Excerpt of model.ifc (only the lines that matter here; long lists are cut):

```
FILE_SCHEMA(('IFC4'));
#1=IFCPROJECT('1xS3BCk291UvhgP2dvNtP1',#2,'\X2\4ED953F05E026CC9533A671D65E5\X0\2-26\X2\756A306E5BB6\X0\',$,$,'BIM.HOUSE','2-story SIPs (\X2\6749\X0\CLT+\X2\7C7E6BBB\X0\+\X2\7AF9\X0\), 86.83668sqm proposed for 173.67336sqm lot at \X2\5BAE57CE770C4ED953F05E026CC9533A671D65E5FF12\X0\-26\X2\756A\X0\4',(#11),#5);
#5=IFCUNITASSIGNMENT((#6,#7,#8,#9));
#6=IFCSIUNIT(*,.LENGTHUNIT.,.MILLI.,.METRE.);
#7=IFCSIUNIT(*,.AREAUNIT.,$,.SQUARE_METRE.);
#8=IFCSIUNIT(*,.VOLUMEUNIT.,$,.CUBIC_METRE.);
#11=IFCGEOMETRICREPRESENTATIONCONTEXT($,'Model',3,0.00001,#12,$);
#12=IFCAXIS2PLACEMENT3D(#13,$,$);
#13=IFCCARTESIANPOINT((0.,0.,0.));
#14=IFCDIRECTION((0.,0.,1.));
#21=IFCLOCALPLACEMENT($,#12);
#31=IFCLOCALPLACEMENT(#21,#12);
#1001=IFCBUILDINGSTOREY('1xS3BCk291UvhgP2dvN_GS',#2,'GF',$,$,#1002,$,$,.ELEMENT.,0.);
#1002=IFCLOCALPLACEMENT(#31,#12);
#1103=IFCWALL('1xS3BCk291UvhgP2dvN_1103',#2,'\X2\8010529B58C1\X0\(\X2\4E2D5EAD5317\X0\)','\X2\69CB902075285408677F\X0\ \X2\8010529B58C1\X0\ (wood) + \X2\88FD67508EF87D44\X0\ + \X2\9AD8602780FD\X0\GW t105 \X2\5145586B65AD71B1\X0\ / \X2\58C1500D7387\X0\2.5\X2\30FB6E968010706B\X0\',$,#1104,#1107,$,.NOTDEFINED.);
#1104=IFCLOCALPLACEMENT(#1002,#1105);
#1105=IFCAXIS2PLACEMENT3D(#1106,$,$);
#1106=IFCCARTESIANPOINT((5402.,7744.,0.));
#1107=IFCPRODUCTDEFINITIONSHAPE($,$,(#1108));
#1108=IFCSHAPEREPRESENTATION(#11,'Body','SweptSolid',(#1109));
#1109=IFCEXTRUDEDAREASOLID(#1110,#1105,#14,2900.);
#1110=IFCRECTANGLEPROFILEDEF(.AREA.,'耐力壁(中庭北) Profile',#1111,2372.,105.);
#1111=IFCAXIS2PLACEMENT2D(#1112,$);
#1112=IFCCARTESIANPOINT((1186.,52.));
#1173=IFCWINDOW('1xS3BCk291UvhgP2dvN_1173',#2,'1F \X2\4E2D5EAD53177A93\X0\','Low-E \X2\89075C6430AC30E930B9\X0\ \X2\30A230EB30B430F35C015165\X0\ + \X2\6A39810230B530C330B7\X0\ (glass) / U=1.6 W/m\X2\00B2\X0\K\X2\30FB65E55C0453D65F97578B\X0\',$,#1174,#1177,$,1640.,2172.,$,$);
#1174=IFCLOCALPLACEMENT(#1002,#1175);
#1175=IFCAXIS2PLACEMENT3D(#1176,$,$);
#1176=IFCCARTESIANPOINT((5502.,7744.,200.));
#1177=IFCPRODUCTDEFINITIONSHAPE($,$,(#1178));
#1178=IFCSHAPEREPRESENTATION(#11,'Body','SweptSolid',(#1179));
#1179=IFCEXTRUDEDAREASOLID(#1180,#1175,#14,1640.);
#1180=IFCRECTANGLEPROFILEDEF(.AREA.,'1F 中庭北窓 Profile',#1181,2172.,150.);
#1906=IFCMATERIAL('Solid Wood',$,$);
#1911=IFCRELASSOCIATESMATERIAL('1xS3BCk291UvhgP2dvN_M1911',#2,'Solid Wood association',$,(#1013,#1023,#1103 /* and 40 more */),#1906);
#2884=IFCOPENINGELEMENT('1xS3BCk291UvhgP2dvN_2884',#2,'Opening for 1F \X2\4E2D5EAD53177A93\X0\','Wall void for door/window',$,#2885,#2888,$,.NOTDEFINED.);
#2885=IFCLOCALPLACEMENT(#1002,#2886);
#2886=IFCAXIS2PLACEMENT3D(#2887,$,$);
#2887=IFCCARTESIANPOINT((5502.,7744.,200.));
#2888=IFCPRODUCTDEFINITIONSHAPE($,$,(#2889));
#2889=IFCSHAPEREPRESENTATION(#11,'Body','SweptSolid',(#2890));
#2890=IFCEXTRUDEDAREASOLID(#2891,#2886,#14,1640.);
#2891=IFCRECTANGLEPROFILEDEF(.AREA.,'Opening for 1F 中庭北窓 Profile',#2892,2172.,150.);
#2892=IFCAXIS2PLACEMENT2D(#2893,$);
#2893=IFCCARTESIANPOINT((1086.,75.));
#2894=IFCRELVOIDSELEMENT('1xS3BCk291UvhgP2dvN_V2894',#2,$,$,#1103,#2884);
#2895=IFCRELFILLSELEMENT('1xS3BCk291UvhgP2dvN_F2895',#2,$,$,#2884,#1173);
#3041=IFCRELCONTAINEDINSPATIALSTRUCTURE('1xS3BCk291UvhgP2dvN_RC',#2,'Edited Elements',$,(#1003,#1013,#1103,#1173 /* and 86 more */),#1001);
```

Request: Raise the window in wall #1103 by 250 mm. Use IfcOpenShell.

```python
import numpy as np
import ifcopenshell
import ifcopenshell.api.geometry
import ifcopenshell.util.placement
import ifcopenshell.util.unit

model = ifcopenshell.open("model.ifc")
unit_scale = ifcopenshell.util.unit.calculate_unit_scale(model)

window = model.by_id(1173)
opening = window.FillsVoids[0].RelatingOpeningElement
dz = 250.0

shift = np.array([0.0, 0.0, dz])
# The window is not placed relative to its opening, so move both.
for product in (opening, window):
    matrix = ifcopenshell.util.placement.get_local_placement(product.ObjectPlacement)
    matrix[:3, 3] += shift
    ifcopenshell.api.geometry.edit_object_placement(model, product=product, matrix=matrix, is_si=False)

print(f"moved by {dz * unit_scale:+.3f} m")

model.write("model_updated.ifc")
```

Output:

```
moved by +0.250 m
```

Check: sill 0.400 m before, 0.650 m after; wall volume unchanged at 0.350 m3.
